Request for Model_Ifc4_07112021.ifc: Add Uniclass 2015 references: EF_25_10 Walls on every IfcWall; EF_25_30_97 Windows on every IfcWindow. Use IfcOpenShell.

First a look at what the model holds.

```python
import ifcopenshell

model = ifcopenshell.open("Model_Ifc4_07112021.ifc")
print(model.schema)
print("classifications:", [c.Name for c in model.by_type("IfcClassification")])
for ifc_class in ("IfcDoor", "IfcRoof", "IfcStair", "IfcWall", "IfcWindow"):
    print(ifc_class, len(model.by_type(ifc_class)))
```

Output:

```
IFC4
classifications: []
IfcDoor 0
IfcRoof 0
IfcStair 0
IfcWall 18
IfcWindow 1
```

```python
import ifcopenshell
import ifcopenshell.api.classification

model = ifcopenshell.open("Model_Ifc4_07112021.ifc")

system = ifcopenshell.api.classification.add_classification(model, classification="Uniclass 2015")

codes = {
    "IfcWall": ("EF_25_10", "Walls"),
    "IfcWindow": ("EF_25_30_97", "Windows"),
}
for ifc_class, (code, name) in codes.items():
    products = model.by_type(ifc_class)
    ifcopenshell.api.classification.add_reference(
        model, products=products, classification=system, identification=code, name=name
    )
    print(code, len(products))

model.write("Model_Ifc4_07112021_updated.ifc")
```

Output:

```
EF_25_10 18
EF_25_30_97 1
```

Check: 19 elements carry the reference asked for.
